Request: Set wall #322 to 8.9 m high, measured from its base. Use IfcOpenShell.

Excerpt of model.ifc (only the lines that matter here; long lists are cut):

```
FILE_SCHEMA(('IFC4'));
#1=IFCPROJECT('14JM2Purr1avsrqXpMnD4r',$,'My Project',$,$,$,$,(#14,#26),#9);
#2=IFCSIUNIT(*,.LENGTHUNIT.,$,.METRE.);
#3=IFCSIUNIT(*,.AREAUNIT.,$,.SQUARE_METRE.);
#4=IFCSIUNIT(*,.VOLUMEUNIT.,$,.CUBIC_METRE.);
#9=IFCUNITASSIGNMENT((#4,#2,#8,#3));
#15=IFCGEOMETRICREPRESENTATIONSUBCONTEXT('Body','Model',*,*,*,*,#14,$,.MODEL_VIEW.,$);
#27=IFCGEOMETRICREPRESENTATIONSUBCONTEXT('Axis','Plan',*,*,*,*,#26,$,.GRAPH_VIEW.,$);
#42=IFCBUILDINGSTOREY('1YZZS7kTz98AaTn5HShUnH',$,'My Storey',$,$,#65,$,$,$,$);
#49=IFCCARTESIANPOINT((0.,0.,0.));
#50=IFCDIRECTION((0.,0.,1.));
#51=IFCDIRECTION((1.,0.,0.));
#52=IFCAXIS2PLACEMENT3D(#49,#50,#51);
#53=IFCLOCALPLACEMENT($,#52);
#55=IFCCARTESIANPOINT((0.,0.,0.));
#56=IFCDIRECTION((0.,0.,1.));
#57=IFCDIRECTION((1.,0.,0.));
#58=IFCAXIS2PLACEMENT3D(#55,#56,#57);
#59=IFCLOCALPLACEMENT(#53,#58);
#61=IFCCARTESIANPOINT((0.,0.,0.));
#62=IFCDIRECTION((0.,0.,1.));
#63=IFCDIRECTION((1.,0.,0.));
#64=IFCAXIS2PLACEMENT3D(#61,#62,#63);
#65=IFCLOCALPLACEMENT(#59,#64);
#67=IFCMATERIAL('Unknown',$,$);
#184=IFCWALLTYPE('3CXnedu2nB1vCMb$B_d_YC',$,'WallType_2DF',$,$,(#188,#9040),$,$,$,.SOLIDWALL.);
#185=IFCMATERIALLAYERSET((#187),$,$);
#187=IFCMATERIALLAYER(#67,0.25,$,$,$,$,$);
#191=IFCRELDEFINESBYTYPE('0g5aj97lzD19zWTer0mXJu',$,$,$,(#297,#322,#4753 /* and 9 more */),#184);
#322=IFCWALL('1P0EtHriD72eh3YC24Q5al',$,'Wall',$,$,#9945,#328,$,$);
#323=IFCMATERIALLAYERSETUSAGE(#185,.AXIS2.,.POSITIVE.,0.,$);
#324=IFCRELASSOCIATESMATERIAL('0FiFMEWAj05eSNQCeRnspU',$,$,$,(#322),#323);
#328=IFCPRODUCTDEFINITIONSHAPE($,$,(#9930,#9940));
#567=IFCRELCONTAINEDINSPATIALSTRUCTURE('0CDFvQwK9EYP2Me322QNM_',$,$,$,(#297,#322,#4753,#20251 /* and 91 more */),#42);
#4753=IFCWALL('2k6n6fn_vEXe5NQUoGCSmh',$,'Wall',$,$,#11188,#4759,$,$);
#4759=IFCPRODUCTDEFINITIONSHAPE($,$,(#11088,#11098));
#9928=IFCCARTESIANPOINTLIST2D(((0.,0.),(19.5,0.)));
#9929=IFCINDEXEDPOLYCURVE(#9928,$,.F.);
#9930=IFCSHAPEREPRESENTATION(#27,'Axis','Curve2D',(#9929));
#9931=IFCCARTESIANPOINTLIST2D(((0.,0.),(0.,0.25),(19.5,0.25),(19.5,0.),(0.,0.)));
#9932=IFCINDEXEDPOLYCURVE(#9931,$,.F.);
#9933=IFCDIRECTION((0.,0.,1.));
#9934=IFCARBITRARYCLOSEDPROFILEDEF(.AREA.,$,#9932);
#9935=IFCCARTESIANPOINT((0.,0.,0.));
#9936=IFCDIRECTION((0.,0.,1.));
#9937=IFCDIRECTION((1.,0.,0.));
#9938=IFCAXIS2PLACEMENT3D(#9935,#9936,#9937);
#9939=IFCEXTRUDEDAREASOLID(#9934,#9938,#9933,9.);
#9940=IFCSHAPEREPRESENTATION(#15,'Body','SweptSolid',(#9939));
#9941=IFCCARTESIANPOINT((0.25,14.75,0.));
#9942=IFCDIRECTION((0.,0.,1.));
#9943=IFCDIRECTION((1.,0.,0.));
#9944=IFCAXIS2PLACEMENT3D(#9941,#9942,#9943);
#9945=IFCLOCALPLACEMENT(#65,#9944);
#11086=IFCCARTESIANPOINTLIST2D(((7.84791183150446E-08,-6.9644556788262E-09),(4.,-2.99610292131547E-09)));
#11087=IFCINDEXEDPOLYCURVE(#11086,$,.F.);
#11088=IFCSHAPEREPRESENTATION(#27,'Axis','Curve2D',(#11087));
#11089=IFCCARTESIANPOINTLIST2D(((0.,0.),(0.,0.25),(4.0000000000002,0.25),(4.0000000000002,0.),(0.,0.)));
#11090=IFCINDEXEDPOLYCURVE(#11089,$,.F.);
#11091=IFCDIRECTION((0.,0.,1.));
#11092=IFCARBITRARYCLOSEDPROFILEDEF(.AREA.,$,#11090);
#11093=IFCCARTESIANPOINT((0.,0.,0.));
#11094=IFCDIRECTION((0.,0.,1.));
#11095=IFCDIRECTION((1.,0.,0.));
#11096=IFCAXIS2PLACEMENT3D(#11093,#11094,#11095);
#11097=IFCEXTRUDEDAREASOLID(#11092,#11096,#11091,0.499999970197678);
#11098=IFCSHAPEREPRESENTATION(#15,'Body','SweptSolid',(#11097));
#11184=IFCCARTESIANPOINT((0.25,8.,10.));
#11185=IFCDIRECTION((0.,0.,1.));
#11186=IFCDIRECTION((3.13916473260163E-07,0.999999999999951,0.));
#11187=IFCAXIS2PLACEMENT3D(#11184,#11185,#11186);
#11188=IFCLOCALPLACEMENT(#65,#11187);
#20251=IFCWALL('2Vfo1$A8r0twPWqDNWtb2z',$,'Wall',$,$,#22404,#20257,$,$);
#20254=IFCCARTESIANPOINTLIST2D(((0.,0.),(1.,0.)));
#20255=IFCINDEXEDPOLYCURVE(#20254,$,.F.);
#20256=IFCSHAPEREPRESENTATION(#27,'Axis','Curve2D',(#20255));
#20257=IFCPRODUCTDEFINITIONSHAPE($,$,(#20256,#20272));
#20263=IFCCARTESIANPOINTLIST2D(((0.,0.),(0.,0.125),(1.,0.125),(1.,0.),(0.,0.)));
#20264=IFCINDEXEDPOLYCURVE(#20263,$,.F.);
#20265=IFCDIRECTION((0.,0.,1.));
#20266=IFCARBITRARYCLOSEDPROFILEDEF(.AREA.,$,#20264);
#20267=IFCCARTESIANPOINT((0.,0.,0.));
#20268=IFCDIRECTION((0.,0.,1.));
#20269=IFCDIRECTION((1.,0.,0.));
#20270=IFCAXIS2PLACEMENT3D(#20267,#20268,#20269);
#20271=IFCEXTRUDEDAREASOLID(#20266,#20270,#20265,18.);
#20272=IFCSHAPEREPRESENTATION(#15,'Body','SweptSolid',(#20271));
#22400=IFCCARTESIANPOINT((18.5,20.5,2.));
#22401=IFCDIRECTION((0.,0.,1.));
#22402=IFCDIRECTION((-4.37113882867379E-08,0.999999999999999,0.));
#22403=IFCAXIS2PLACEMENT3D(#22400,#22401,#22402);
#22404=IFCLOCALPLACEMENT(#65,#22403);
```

```python
import ifcopenshell
import ifcopenshell.geom
import ifcopenshell.util.representation
import ifcopenshell.util.shape

model = ifcopenshell.open("model.ifc")
settings = ifcopenshell.geom.settings()


def volume(element):
    """Net volume in cubic metres, openings subtracted."""
    shape = ifcopenshell.geom.create_shape(settings, element)
    return ifcopenshell.util.shape.get_volume(shape.geometry)


wall = model.by_guid("1P0EtHriD72eh3YC24Q5al")
before = volume(wall)

body = ifcopenshell.util.representation.get_representation(wall, "Model", "Body")
solid = body.Items[0]
old_height = solid.Depth
solid.Depth = 8.9
after = volume(wall)

print(f"height {old_height:g} -> {solid.Depth:g}, volume {before:.3f} -> {after:.3f} m3")

model.write("model_rev.ifc")
```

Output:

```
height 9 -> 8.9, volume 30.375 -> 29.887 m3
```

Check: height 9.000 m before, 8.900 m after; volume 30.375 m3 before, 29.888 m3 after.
